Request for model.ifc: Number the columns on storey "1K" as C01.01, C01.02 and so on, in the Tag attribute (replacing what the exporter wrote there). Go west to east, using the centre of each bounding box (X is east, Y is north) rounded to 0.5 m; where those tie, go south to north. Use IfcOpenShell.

First a look at what the model holds.

```python
import ifcopenshell
import ifcopenshell.util.element
import ifcopenshell.util.placement

model = ifcopenshell.open("model.ifc")
print(model.schema)
storey = next(s for s in model.by_type("IfcBuildingStorey") if s.Name == '1\x8aK')
columns = [e for e in ifcopenshell.util.element.get_decomposition(storey) if e.is_a("IfcColumn")]
for e in sorted(columns, key=lambda e: e.id()):
    origin = ifcopenshell.util.placement.get_local_placement(e.ObjectPlacement)[:3, 3]
    print(e.id(), e.Tag, e.Name, origin.round(2) + 0.0, sep=" | ")
```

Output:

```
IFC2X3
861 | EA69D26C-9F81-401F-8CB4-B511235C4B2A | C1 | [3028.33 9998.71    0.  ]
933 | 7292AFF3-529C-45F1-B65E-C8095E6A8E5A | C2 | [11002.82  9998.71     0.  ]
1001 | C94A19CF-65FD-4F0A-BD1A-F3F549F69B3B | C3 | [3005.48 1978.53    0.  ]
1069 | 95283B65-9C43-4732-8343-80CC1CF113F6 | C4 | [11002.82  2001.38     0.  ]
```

```python
import ifcopenshell
import ifcopenshell.geom
import ifcopenshell.util.element
import ifcopenshell.util.shape

model = ifcopenshell.open("model.ifc")
settings = ifcopenshell.geom.settings()
settings.set("use-world-coords", True)


def centre(element):
    shape = ifcopenshell.geom.create_shape(settings, element)
    return ifcopenshell.util.shape.get_bbox_centroid(shape.geometry)


storey = next(s for s in model.by_type("IfcBuildingStorey") if s.Name == '1\x8aK')
columns = [e for e in ifcopenshell.util.element.get_decomposition(storey) if e.is_a("IfcColumn")]

# Insertion points can sit at a corner or the storey origin, so sort by the geometry (in metres).
centres = {e: centre(e) for e in columns}
columns.sort(key=lambda e: (round(centres[e][0] / 0.5), centres[e][1]))

for i, e in enumerate(columns, start=1):
    number = f"C01.{i:02d}"
    e.Tag = number
    print(e.id(), number)

model.write("model_rev.ifc")
```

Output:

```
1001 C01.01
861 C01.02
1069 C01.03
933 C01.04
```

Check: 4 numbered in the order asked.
